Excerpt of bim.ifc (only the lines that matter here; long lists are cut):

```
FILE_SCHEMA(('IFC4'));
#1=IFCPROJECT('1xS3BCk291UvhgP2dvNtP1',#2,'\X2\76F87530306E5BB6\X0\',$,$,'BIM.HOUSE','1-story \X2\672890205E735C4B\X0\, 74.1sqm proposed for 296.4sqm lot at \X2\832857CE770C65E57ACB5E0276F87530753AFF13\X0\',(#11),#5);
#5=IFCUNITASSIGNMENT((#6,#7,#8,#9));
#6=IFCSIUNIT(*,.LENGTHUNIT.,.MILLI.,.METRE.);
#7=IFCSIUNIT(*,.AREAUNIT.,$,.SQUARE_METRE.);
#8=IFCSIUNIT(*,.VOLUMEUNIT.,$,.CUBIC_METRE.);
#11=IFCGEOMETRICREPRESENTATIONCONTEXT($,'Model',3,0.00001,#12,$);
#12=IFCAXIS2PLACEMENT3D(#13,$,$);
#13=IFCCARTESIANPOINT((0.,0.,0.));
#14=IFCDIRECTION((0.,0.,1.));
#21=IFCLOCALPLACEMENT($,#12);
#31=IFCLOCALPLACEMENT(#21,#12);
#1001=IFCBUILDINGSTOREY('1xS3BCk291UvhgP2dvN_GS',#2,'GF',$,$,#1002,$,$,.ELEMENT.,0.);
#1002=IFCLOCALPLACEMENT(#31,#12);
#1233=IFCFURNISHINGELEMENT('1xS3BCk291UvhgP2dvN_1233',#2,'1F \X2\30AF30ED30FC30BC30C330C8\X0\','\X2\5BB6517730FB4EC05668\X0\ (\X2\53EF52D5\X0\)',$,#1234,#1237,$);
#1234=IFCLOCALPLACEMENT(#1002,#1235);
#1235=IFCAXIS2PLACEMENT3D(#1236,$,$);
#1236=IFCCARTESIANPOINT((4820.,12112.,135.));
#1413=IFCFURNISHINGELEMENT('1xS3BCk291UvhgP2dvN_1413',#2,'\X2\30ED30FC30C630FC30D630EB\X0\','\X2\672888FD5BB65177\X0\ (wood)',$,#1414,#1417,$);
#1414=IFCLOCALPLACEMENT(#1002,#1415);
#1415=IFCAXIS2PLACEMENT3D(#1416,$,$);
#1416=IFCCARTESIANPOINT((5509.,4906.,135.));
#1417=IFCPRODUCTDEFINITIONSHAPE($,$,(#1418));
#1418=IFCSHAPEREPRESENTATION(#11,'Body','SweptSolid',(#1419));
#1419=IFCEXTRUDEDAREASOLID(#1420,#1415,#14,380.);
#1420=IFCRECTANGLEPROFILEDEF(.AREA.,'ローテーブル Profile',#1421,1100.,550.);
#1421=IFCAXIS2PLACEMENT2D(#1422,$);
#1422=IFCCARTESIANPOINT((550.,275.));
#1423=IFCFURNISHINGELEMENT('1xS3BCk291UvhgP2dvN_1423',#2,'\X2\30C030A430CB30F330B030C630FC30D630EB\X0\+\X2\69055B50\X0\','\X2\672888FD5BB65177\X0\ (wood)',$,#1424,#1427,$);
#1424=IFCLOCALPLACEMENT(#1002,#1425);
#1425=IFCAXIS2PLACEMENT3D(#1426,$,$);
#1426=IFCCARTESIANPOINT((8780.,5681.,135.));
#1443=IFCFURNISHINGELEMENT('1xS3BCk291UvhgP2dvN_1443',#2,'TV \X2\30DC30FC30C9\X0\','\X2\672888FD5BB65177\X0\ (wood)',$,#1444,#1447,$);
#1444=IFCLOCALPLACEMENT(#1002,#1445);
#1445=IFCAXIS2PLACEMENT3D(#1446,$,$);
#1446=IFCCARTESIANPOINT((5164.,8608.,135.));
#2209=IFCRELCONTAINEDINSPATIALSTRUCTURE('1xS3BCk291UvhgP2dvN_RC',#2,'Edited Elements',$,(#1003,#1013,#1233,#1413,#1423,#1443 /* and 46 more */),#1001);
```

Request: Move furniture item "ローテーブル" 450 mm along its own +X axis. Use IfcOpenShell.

```python
import ifcopenshell
import ifcopenshell.api.geometry
import ifcopenshell.util.placement

model = ifcopenshell.open("bim.ifc")

item = model.by_guid("1xS3BCk291UvhgP2dvN_1413")
matrix = ifcopenshell.util.placement.get_local_placement(item.ObjectPlacement)
matrix[:3, 3] += matrix[:3, 0] * 450.0
ifcopenshell.api.geometry.edit_object_placement(model, product=item, matrix=matrix, is_si=False)

print(ifcopenshell.util.placement.get_local_placement(item.ObjectPlacement).round(3) + 0.0)

model.write("bim_rev.ifc")
```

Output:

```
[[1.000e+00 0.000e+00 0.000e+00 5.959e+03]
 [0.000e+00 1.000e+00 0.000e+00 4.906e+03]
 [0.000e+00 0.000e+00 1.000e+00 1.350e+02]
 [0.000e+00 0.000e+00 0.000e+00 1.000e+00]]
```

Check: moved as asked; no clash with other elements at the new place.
